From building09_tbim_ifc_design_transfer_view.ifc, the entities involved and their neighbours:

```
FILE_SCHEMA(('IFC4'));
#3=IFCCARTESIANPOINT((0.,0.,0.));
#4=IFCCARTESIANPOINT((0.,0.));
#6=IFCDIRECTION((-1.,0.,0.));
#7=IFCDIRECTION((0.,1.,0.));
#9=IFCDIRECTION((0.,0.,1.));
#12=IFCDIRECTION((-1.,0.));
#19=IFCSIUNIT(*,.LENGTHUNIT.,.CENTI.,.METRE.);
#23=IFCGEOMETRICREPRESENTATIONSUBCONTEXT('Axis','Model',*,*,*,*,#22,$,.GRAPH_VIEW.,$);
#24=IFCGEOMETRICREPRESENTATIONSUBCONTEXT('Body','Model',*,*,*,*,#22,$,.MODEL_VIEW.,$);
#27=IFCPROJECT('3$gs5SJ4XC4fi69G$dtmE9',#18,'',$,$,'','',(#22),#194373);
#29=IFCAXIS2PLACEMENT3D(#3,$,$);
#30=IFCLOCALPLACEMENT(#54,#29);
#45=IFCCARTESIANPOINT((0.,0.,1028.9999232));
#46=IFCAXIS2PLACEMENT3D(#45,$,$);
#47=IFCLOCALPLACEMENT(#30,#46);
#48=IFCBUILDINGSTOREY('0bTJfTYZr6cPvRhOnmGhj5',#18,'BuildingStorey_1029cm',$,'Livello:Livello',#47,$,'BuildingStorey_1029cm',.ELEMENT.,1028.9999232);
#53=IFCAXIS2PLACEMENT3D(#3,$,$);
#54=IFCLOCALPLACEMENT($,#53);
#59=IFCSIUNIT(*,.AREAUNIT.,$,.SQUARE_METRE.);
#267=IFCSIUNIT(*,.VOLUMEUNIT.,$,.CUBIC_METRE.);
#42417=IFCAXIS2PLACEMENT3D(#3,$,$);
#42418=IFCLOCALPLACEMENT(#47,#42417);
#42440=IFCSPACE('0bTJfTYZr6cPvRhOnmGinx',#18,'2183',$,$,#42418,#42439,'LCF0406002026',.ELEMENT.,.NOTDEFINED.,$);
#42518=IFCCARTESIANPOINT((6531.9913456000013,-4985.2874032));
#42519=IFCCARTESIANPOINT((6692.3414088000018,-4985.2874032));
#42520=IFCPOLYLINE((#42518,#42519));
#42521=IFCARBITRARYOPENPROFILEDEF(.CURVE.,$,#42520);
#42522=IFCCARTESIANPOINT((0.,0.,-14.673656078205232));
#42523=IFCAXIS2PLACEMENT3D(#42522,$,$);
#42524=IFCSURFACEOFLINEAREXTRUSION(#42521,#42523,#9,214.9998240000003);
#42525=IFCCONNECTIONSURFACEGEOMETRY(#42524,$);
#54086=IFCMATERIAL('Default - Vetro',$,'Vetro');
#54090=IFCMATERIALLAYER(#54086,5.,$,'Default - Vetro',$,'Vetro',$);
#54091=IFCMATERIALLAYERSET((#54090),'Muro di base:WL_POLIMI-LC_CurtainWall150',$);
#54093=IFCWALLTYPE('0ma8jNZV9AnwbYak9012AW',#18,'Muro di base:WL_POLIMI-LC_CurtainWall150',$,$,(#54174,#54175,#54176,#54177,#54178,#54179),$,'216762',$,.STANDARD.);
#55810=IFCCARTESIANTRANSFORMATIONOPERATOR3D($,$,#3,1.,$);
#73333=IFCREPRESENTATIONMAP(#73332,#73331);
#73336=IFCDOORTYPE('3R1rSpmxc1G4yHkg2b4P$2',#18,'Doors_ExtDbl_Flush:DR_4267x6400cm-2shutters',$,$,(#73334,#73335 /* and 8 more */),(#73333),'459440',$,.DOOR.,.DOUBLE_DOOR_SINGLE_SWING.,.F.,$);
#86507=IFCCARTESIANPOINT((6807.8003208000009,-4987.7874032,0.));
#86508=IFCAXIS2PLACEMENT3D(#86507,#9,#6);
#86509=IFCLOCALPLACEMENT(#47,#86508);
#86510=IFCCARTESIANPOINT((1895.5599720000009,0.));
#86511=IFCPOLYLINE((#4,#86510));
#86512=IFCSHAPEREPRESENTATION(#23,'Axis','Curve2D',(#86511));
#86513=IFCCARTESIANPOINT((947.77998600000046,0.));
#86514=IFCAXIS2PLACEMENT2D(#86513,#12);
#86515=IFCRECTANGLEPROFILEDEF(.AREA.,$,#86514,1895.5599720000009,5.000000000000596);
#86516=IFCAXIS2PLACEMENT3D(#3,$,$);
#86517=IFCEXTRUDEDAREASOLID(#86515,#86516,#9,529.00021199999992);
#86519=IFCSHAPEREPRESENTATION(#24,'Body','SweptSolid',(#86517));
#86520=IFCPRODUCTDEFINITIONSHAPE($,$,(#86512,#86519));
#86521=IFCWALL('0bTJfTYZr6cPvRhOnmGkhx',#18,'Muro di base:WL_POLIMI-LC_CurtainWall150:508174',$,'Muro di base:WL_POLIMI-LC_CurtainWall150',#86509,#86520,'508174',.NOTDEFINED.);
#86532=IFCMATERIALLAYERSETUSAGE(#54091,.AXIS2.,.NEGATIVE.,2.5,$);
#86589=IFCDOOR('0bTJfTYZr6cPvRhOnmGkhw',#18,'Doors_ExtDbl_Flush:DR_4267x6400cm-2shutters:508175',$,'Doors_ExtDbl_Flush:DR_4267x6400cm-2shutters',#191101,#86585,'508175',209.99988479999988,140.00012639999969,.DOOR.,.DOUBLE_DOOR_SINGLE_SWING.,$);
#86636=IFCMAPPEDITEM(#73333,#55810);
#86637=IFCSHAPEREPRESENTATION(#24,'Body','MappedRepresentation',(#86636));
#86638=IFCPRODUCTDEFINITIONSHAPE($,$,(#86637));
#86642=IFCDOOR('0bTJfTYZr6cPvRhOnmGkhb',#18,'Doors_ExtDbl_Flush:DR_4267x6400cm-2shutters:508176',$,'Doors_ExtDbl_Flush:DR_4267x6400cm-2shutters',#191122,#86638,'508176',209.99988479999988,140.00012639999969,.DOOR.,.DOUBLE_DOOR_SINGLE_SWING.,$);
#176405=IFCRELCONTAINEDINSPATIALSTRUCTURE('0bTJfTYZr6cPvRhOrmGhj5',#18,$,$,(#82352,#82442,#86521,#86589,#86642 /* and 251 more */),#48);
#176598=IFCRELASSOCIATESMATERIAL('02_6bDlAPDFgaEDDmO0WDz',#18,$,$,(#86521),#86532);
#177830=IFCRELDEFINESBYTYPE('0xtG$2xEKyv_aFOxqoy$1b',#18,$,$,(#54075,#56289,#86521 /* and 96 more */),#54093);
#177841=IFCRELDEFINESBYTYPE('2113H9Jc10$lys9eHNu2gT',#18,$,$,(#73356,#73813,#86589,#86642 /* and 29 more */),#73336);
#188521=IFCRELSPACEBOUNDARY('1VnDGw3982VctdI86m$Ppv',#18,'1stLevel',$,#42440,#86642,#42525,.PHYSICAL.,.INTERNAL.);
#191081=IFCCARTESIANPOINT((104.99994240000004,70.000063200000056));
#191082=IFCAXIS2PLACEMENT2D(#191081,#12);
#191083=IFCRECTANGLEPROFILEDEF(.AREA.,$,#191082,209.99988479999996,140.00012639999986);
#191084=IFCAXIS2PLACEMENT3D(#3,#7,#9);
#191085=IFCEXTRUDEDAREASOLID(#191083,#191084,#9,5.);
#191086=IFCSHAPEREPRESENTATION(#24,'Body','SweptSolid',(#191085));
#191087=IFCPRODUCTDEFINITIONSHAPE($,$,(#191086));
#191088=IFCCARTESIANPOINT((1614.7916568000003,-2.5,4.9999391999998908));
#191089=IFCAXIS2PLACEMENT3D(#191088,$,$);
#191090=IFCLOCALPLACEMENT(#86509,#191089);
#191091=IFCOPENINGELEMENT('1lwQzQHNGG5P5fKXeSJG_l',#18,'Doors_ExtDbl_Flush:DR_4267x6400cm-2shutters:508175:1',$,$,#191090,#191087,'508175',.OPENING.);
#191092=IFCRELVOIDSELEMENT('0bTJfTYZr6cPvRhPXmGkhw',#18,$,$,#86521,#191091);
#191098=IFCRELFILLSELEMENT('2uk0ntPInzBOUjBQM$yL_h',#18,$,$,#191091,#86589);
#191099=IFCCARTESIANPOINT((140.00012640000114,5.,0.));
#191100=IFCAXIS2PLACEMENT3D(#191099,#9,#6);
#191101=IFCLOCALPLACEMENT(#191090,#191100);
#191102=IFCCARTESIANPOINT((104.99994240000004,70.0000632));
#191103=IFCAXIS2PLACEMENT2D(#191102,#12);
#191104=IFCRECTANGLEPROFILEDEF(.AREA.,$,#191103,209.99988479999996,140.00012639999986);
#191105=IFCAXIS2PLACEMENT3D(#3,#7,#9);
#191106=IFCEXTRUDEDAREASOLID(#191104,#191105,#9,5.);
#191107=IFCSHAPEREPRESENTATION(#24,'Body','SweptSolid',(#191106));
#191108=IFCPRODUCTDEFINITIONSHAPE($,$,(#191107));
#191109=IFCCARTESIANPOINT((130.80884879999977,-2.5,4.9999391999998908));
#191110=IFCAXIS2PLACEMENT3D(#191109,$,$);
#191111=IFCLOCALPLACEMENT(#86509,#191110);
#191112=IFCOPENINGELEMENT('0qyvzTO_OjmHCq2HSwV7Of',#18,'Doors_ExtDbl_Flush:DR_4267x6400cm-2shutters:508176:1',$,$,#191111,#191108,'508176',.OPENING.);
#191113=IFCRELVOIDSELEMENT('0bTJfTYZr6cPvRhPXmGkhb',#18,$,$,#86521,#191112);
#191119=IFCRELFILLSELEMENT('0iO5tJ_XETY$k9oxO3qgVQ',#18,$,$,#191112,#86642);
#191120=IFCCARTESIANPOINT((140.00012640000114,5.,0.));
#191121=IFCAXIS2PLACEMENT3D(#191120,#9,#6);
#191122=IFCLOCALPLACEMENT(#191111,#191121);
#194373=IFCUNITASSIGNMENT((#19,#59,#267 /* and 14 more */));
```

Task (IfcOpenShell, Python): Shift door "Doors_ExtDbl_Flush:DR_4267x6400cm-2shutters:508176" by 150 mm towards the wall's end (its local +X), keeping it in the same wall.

```python
import numpy as np
import ifcopenshell
import ifcopenshell.api.geometry
import ifcopenshell.util.placement
import ifcopenshell.util.unit

model = ifcopenshell.open("building09_tbim_ifc_design_transfer_view.ifc")
unit_scale = ifcopenshell.util.unit.calculate_unit_scale(model)

door = model.by_id(86642)
opening = door.FillsVoids[0].RelatingOpeningElement
wall = opening.VoidsElements[0].RelatingBuildingElement

wall_matrix = ifcopenshell.util.placement.get_local_placement(wall.ObjectPlacement)
shift = wall_matrix[:3, 0] * 0.15 / unit_scale
before = ifcopenshell.util.placement.get_local_placement(door.ObjectPlacement)[:3, 3].copy()

# The door is placed relative to its opening, so it follows when the opening moves.
matrix = ifcopenshell.util.placement.get_local_placement(opening.ObjectPlacement)
matrix[:3, 3] += shift
ifcopenshell.api.geometry.edit_object_placement(
    model, product=opening, matrix=matrix, is_si=False, should_transform_children=True
)

# Space boundary surfaces are stored in each space's coordinates; move them too.
for rel in door.ProvidesBoundaries:
    if not rel.ConnectionGeometry:
        continue
    surface = rel.ConnectionGeometry.SurfaceOnRelatingElement
    space_matrix = ifcopenshell.util.placement.get_local_placement(rel.RelatingSpace.ObjectPlacement)
    point = np.array(surface.Position.Location.Coordinates) + space_matrix[:3, :3].T @ shift
    surface.Position = model.createIfcAxis2Placement3D(
        model.createIfcCartesianPoint(point.tolist()), surface.Position.Axis, surface.Position.RefDirection
    )

after = ifcopenshell.util.placement.get_local_placement(door.ObjectPlacement)[:3, 3]
print("door moved by", (after - before).round(3) + 0.0)

model.write("building09_tbim_ifc_design_transfer_view_updated.ifc")
```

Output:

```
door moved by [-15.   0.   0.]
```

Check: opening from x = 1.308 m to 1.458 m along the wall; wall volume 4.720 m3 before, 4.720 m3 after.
